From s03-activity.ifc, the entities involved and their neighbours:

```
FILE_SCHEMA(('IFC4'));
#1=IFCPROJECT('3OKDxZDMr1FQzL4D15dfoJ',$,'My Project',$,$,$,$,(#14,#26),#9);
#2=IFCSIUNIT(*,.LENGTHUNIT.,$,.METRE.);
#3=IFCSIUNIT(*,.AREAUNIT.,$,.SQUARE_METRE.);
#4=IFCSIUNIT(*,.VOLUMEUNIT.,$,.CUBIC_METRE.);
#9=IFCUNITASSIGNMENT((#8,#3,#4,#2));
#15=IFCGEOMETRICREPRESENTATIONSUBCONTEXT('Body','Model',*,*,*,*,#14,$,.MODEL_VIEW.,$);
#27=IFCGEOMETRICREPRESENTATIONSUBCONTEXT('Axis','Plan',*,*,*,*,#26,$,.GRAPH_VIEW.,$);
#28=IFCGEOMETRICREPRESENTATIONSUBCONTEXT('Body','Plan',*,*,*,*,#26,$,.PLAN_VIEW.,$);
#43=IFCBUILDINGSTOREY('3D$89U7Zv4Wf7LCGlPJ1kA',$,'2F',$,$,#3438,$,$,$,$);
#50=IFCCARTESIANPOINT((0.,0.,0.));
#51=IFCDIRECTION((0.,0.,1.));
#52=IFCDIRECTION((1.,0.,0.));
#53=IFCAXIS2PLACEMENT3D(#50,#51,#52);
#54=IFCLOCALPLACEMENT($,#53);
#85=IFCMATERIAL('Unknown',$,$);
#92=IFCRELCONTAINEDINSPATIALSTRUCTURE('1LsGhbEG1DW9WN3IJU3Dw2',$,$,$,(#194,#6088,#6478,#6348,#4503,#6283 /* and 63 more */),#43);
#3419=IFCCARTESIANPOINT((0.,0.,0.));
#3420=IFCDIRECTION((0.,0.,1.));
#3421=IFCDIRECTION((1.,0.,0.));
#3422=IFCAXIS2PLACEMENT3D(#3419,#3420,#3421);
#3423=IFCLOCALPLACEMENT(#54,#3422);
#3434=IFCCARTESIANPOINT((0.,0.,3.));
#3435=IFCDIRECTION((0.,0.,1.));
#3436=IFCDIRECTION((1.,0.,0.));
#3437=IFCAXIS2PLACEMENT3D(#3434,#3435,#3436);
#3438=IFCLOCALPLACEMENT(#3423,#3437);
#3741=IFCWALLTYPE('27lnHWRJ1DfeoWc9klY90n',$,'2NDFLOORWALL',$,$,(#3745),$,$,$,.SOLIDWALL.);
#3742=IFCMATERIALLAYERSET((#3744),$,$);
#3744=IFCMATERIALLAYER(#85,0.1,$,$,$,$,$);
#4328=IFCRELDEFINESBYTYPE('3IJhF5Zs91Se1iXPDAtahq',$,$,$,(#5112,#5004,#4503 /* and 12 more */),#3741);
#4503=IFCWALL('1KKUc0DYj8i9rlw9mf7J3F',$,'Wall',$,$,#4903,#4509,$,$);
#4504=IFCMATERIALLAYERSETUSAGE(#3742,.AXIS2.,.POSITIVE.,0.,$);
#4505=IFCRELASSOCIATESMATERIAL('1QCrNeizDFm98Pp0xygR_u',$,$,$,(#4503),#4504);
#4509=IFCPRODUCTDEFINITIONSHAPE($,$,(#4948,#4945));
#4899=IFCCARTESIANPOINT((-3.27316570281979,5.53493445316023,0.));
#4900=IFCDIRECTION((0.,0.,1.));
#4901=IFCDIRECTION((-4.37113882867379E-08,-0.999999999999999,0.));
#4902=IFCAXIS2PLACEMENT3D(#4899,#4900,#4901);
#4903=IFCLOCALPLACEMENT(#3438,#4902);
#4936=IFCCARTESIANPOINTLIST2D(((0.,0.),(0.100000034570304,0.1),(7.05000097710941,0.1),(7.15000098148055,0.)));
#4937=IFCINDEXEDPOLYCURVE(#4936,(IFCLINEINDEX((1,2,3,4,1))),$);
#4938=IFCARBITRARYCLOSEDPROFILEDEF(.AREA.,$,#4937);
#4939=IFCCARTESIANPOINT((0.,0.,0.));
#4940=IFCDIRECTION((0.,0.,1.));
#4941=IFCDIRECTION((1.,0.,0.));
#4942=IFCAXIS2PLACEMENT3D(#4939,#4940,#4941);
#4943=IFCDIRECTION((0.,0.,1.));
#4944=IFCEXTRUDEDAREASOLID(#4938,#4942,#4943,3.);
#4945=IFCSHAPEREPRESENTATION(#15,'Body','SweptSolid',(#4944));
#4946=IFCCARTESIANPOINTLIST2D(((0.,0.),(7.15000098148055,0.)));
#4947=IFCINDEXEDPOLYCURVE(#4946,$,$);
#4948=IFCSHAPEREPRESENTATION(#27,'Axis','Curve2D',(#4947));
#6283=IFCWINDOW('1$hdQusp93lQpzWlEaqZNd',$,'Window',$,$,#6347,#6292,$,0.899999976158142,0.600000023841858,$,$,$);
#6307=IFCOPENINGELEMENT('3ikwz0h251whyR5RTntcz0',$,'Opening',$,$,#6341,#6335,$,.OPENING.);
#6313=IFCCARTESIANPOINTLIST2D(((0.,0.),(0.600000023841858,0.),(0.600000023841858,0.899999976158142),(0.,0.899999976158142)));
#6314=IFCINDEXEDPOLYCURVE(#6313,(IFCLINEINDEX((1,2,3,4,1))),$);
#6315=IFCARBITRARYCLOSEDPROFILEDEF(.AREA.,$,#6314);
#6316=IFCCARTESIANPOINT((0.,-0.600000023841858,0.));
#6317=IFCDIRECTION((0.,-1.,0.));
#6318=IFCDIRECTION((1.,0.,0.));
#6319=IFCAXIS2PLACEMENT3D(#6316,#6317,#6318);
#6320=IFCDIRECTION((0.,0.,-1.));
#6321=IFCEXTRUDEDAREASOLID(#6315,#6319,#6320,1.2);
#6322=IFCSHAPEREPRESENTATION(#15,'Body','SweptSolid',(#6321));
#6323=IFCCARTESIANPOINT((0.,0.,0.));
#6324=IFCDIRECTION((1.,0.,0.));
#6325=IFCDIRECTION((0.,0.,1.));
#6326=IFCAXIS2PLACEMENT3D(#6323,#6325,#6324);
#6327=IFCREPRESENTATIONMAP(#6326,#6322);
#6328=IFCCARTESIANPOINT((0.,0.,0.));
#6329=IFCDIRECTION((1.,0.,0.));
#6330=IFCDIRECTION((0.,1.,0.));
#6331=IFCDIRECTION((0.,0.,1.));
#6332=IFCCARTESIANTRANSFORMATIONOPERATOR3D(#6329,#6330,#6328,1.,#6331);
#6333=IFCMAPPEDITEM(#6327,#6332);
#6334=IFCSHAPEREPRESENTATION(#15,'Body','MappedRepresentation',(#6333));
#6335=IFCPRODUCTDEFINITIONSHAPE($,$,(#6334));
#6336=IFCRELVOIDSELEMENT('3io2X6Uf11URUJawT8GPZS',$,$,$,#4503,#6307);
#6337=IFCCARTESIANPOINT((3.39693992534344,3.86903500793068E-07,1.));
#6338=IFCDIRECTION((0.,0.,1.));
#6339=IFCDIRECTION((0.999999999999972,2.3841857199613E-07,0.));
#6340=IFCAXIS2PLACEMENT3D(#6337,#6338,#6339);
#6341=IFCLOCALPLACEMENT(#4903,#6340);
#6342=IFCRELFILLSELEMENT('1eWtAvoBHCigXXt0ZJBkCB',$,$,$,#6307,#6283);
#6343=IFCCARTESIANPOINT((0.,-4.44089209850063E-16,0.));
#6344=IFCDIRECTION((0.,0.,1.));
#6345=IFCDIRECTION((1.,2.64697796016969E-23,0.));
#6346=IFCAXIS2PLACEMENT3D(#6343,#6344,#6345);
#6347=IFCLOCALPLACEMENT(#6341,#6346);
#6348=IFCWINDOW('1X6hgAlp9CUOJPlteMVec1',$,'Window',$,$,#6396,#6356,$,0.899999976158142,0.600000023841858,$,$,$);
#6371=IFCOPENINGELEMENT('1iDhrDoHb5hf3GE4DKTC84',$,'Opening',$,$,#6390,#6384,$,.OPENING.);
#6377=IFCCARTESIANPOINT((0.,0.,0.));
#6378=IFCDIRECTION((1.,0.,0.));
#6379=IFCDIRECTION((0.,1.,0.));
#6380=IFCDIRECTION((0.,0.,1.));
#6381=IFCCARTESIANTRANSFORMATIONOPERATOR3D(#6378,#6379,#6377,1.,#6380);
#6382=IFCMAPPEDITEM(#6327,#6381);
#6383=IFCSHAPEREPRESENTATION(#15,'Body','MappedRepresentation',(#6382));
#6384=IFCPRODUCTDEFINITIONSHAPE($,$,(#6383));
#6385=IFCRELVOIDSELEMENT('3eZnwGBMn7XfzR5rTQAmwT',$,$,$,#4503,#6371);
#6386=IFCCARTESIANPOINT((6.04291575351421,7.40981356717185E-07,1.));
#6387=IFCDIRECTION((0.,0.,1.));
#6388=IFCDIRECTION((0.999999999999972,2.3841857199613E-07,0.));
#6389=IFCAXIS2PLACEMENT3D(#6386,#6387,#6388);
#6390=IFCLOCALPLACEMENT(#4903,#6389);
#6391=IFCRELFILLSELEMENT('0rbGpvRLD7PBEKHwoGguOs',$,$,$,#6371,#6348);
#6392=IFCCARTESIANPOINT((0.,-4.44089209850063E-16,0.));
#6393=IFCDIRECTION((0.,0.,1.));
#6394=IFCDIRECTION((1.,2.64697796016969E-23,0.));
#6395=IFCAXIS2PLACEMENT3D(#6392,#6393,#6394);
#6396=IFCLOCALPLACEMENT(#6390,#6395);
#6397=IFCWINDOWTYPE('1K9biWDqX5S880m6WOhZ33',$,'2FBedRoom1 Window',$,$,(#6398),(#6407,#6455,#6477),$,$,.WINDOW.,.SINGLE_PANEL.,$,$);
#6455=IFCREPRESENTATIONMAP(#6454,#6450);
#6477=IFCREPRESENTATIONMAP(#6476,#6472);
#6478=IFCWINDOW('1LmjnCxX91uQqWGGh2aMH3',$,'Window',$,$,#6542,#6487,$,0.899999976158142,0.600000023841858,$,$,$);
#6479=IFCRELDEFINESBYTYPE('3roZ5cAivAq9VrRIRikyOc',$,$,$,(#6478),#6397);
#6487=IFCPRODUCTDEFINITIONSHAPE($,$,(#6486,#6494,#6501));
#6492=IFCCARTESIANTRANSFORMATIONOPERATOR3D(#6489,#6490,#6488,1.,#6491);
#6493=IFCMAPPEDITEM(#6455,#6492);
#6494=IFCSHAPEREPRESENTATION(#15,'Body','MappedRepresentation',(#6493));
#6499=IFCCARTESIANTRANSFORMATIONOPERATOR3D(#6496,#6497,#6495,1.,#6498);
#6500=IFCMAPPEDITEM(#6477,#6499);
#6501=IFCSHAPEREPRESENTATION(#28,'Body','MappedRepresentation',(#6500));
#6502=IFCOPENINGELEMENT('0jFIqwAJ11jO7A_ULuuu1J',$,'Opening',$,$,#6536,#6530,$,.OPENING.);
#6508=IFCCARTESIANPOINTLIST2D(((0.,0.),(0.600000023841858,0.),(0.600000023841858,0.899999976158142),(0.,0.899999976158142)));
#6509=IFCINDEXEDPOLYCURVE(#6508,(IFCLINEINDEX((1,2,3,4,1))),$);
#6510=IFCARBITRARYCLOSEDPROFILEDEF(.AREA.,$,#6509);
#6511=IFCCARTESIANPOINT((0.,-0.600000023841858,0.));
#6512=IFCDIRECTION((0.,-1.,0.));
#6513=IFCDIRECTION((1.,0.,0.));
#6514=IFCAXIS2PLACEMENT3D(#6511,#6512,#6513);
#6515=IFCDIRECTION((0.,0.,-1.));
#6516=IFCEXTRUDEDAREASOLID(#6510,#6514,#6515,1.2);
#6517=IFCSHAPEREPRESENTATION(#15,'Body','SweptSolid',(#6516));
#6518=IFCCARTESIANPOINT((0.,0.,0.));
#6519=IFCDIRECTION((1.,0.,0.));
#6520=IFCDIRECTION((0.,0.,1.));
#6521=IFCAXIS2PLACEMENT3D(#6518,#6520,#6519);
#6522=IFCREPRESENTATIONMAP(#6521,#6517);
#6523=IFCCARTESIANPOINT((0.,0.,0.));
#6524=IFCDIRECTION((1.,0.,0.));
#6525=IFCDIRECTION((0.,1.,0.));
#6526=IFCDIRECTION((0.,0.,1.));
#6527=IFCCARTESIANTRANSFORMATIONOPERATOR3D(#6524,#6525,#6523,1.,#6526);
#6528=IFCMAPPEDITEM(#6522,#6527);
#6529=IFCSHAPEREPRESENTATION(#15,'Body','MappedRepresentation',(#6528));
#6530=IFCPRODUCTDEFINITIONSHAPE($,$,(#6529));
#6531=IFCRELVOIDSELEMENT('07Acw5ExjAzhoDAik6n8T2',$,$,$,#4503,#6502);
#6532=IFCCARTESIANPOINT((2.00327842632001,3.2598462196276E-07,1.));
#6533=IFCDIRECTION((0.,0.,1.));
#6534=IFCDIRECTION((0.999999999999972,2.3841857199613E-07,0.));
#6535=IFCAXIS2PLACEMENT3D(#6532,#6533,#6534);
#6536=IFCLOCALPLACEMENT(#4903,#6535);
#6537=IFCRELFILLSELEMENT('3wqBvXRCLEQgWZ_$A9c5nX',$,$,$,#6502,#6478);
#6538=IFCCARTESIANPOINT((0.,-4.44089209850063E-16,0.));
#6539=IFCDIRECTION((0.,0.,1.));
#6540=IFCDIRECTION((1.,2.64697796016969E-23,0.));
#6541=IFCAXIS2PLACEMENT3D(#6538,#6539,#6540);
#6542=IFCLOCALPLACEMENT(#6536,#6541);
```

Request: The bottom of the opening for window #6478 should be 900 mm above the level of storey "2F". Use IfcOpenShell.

```python
import numpy as np
import ifcopenshell
import ifcopenshell.api.geometry
import ifcopenshell.geom
import ifcopenshell.util.element
import ifcopenshell.util.placement
import ifcopenshell.util.shape
import ifcopenshell.util.unit

model = ifcopenshell.open("s03-activity.ifc")
unit_scale = ifcopenshell.util.unit.calculate_unit_scale(model)

window = model.by_guid("1LmjnCxX91uQqWGGh2aMH3")
opening = window.FillsVoids[0].RelatingOpeningElement
storey = ifcopenshell.util.element.get_container(window, ifc_class="IfcBuildingStorey")
level = ifcopenshell.util.placement.get_local_placement(storey.ObjectPlacement)[2, 3]

# The opening's origin need not be at the sill, so measure its lowest point.
shape = ifcopenshell.geom.create_shape(ifcopenshell.geom.settings(), opening)
bottom = ifcopenshell.util.shape.get_shape_bottom_elevation(shape, shape.geometry) / unit_scale
dz = level + 0.9 / unit_scale - bottom

shift = np.array([0.0, 0.0, dz])
# The window is placed relative to its opening, so it follows when the opening moves.
matrix = ifcopenshell.util.placement.get_local_placement(opening.ObjectPlacement)
matrix[:3, 3] += shift
ifcopenshell.api.geometry.edit_object_placement(
    model, product=opening, matrix=matrix, is_si=False, should_transform_children=True
)

print(f"moved by {dz * unit_scale:+.3f} m")

model.write("s03-activity_rev.ifc")
```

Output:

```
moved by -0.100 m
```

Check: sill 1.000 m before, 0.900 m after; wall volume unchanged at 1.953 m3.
